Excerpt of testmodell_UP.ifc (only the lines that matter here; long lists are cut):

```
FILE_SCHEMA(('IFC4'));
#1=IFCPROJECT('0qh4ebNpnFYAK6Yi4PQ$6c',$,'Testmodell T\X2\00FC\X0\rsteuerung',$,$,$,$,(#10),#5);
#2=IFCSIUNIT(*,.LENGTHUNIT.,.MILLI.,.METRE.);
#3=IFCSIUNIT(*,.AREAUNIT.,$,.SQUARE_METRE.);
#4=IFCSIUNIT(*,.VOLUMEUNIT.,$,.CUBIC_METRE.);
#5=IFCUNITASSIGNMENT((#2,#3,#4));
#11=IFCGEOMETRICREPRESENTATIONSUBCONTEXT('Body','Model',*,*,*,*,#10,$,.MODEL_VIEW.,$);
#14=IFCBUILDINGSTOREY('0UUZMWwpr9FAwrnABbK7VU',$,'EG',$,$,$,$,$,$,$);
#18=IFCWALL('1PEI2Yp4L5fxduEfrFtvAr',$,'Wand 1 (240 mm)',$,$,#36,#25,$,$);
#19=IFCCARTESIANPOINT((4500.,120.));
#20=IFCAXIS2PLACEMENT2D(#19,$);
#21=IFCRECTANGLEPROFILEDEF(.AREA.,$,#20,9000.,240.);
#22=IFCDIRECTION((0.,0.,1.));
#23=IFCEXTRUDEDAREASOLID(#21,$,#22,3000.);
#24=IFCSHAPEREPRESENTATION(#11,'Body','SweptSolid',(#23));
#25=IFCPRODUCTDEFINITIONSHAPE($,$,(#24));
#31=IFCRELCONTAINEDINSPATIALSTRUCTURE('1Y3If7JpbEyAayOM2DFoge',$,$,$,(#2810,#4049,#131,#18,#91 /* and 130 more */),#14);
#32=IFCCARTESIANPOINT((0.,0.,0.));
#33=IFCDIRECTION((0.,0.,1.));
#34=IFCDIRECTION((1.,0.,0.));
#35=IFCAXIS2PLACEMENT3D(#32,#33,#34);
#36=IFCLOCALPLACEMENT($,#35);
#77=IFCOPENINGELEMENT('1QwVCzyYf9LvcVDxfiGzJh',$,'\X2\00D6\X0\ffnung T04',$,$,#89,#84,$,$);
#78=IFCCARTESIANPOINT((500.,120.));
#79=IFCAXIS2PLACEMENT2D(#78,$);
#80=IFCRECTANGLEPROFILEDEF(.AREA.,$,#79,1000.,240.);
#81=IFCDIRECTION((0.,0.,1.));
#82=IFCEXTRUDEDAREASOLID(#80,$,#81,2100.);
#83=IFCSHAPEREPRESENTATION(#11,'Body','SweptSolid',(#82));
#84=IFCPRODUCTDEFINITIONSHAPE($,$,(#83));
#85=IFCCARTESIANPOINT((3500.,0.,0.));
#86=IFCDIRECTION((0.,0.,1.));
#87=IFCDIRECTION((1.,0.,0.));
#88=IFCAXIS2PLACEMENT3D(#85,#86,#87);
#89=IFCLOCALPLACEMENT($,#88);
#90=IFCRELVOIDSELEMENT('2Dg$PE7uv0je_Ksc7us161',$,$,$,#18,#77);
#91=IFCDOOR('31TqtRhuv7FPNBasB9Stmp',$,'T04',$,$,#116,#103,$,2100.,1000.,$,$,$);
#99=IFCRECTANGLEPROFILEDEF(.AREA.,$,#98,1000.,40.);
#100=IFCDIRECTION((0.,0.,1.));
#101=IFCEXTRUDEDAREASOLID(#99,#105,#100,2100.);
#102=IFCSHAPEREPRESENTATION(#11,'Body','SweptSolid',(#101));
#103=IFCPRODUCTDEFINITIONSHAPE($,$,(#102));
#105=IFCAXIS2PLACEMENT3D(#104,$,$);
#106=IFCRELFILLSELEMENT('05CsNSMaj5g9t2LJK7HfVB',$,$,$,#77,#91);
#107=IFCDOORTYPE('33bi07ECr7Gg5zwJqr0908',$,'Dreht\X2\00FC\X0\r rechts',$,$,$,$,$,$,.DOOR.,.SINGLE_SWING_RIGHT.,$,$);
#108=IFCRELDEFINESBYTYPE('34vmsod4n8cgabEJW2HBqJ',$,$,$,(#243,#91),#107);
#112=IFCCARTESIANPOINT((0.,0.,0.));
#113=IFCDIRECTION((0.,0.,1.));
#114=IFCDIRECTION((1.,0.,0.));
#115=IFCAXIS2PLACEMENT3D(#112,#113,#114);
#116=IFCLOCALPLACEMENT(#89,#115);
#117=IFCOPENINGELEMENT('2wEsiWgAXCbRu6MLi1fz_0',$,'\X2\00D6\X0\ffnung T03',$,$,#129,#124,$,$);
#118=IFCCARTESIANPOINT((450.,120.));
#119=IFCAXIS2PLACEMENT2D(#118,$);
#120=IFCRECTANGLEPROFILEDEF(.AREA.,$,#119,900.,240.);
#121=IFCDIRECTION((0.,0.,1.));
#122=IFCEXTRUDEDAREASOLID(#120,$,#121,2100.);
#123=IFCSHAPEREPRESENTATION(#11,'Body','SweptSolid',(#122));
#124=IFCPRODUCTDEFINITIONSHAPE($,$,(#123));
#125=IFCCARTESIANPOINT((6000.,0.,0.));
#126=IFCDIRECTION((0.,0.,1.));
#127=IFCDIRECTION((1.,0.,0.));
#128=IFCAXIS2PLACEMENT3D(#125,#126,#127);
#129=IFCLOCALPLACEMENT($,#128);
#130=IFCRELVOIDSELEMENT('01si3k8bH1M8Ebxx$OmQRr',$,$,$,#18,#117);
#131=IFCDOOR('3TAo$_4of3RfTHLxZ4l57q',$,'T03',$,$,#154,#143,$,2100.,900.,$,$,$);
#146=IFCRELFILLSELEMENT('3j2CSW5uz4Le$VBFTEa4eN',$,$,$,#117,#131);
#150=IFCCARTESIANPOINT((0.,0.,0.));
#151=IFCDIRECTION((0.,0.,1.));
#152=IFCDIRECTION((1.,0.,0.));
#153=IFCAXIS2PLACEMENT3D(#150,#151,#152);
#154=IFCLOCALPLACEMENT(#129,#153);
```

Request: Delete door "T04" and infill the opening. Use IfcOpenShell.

```python
import ifcopenshell
import ifcopenshell.api.feature
import ifcopenshell.api.root
import ifcopenshell.geom
import ifcopenshell.util.shape

model = ifcopenshell.open("testmodell_UP.ifc")
settings = ifcopenshell.geom.settings()


def volume(element):
    """Net volume in cubic metres, openings subtracted."""
    shape = ifcopenshell.geom.create_shape(settings, element)
    return ifcopenshell.util.shape.get_volume(shape.geometry)


door = model.by_guid("31TqtRhuv7FPNBasB9Stmp")
opening = door.FillsVoids[0].RelatingOpeningElement
wall = opening.VoidsElements[0].RelatingBuildingElement
before = volume(wall)

ifcopenshell.api.root.remove_product(model, product=door)
ifcopenshell.api.feature.remove_feature(model, feature=opening)

after = volume(wall)

print(f"wall volume {before:.3f} -> {after:.3f} m3")

model.write("testmodell_UP-out.ifc")
```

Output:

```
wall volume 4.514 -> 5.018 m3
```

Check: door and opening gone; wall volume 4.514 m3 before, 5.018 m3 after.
